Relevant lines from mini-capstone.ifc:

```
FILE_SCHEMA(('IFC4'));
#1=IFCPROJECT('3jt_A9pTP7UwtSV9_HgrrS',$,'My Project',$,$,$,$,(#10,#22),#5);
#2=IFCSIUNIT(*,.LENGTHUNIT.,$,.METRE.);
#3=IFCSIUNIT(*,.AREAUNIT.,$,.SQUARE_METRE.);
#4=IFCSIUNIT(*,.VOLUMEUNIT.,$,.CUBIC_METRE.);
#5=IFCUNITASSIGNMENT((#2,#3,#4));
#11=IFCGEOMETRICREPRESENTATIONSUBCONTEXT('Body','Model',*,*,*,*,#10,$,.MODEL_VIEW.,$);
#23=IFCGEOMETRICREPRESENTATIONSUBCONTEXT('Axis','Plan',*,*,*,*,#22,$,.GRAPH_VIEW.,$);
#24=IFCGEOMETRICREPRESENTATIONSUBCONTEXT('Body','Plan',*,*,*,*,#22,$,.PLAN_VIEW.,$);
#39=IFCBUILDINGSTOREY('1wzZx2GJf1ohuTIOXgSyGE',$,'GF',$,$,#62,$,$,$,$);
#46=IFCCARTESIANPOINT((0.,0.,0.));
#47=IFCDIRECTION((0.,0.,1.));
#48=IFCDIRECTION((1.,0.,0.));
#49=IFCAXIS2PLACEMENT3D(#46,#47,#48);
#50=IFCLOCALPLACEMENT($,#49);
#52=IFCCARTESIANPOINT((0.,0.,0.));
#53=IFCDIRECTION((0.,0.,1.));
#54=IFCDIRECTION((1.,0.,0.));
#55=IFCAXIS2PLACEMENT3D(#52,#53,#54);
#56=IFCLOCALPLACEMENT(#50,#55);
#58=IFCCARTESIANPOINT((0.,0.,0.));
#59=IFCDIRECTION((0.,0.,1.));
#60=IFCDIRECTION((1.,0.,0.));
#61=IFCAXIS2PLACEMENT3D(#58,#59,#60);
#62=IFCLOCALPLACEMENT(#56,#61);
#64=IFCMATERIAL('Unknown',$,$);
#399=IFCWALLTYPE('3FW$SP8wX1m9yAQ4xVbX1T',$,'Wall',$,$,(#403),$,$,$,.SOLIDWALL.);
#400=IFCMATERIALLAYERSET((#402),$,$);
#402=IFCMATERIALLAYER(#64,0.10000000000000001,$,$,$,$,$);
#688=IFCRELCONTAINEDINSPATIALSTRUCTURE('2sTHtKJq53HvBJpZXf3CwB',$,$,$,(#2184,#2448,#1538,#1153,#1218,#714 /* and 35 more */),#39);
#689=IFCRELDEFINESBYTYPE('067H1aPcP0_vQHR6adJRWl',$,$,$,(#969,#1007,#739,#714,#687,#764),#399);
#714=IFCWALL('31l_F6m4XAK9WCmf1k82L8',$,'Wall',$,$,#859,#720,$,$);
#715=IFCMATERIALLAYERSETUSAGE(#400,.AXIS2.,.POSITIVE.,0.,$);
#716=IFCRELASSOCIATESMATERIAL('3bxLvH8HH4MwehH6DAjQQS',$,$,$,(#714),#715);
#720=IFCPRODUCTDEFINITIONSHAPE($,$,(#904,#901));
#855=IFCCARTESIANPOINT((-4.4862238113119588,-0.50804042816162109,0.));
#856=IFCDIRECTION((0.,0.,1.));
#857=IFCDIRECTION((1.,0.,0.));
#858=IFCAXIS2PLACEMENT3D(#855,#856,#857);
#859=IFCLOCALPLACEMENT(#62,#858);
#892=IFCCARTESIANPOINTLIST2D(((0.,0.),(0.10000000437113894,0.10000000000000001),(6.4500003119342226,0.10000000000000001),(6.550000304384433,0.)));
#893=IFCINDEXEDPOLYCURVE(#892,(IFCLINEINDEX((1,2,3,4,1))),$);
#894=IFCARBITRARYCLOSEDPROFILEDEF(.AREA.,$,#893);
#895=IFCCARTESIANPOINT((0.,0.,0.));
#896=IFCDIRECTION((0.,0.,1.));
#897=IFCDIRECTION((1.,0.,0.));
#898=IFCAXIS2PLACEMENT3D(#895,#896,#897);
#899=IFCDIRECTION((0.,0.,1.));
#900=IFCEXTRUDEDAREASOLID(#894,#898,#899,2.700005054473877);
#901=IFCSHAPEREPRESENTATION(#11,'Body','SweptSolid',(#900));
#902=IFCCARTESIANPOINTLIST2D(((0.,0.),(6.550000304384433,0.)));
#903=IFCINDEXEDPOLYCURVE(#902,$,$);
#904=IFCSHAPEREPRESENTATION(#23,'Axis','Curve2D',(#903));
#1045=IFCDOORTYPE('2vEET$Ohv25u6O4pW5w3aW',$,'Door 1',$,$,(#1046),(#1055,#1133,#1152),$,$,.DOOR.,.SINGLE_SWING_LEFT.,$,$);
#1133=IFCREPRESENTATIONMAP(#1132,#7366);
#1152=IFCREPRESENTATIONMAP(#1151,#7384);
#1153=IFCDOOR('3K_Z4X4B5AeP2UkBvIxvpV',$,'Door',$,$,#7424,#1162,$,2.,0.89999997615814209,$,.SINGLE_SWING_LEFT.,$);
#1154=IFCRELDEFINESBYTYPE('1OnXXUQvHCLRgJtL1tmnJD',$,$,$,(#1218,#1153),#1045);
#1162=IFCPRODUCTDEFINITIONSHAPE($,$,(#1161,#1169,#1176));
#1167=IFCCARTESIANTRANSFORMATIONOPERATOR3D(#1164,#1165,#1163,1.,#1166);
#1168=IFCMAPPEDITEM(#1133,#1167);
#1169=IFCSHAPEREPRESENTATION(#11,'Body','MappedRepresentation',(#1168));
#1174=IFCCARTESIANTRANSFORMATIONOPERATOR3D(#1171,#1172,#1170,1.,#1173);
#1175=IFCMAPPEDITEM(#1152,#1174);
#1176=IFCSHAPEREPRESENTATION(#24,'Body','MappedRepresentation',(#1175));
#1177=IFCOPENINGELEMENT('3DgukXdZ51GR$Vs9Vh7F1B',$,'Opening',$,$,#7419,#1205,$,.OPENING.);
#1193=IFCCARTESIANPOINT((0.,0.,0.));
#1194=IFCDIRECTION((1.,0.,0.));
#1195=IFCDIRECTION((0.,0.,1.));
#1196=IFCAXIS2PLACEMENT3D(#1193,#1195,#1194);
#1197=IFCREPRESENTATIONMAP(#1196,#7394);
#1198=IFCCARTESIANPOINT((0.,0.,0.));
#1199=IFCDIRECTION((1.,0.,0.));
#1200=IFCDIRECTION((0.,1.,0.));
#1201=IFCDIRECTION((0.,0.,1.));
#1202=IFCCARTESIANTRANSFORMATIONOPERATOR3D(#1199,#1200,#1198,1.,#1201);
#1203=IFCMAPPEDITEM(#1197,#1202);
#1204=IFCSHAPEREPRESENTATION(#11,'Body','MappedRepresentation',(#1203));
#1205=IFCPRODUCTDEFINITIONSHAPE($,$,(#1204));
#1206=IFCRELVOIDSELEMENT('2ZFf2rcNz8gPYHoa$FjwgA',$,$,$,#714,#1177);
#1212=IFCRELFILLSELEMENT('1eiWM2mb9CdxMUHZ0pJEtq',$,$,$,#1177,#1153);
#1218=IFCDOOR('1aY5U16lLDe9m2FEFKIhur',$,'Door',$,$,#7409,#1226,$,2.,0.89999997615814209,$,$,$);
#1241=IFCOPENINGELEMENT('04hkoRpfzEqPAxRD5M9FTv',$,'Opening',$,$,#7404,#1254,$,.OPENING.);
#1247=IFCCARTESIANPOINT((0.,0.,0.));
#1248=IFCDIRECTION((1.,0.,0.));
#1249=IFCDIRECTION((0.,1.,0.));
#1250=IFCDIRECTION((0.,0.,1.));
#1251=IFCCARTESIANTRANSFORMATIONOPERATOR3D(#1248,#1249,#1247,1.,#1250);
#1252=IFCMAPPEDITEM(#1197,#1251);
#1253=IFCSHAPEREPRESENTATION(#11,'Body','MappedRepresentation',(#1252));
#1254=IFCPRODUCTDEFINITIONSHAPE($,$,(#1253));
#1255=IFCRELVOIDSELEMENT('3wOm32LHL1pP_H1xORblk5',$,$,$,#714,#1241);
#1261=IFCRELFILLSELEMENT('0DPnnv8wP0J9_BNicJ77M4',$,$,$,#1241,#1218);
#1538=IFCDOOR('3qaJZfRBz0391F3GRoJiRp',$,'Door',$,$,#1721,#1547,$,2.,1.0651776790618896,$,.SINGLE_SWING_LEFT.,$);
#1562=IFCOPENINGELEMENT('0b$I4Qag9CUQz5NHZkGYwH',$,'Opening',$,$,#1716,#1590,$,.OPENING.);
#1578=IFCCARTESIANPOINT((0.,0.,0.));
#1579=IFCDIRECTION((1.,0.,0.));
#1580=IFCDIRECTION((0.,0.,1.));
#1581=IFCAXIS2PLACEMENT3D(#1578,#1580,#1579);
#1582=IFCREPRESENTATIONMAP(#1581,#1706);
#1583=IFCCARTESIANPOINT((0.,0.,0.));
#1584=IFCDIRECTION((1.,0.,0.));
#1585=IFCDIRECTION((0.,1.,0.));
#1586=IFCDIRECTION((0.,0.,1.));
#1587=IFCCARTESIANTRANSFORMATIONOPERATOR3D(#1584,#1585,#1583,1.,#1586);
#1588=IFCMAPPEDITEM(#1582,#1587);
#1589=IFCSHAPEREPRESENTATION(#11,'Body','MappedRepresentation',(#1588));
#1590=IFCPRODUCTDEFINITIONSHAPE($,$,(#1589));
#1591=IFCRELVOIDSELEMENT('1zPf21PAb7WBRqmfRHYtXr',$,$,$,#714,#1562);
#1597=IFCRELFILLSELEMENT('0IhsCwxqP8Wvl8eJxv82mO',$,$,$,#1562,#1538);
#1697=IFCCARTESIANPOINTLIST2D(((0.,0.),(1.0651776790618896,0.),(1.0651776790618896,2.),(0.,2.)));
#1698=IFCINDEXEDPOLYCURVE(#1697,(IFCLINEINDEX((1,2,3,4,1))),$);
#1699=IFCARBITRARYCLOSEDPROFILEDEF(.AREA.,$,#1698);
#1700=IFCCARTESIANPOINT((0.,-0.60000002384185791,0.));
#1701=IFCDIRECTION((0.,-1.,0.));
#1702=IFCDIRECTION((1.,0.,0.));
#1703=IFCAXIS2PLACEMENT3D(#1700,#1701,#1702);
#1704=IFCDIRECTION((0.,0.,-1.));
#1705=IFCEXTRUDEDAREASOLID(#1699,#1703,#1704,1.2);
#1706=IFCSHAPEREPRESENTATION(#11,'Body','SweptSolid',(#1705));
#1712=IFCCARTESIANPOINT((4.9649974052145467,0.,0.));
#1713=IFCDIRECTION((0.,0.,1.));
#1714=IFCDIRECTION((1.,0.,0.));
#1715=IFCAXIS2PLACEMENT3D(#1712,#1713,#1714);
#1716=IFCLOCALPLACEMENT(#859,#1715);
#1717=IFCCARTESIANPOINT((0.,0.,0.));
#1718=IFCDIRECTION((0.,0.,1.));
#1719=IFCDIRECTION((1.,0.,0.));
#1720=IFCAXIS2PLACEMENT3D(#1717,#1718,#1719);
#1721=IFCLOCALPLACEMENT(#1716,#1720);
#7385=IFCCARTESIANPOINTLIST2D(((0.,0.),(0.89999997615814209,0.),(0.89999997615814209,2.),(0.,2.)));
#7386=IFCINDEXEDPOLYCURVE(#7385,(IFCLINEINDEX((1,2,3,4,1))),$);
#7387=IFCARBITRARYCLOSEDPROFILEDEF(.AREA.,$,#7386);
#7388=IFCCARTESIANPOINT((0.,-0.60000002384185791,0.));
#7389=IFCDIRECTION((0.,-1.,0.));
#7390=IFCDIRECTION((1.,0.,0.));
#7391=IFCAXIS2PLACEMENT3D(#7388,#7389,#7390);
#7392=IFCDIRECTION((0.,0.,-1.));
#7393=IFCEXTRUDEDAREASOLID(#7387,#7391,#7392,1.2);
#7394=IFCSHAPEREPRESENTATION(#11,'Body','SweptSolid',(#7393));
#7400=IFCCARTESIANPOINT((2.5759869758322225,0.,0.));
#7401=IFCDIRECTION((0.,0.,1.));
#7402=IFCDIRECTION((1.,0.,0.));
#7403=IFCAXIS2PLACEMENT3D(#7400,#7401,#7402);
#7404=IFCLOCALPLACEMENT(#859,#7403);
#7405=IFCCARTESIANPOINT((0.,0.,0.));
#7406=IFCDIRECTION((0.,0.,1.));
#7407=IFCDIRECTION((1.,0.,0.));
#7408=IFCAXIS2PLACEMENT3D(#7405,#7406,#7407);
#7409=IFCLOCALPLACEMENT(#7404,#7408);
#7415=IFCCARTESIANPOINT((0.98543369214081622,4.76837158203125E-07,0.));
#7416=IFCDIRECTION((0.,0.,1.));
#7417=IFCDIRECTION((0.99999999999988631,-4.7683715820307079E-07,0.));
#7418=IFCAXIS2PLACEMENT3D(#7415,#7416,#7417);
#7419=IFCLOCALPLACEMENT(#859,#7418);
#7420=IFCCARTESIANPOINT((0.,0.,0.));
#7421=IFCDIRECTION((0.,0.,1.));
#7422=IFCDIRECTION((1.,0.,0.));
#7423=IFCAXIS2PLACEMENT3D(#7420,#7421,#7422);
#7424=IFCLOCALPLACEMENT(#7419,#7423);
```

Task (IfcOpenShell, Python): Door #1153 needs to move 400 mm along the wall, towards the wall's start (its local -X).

```python
import ifcopenshell
import ifcopenshell.api.geometry
import ifcopenshell.util.placement
import ifcopenshell.util.unit

model = ifcopenshell.open("mini-capstone.ifc")
unit_scale = ifcopenshell.util.unit.calculate_unit_scale(model)

door = model.by_guid("3K_Z4X4B5AeP2UkBvIxvpV")
opening = door.FillsVoids[0].RelatingOpeningElement
wall = opening.VoidsElements[0].RelatingBuildingElement

wall_matrix = ifcopenshell.util.placement.get_local_placement(wall.ObjectPlacement)
shift = wall_matrix[:3, 0] * -0.4 / unit_scale
before = ifcopenshell.util.placement.get_local_placement(door.ObjectPlacement)[:3, 3].copy()

# The door is placed relative to its opening, so it follows when the opening moves.
matrix = ifcopenshell.util.placement.get_local_placement(opening.ObjectPlacement)
matrix[:3, 3] += shift
ifcopenshell.api.geometry.edit_object_placement(
    model, product=opening, matrix=matrix, is_si=False, should_transform_children=True
)

after = ifcopenshell.util.placement.get_local_placement(door.ObjectPlacement)[:3, 3]
print("door moved by", (after - before).round(3) + 0.0)

model.write("mini-capstone-out.ifc")
```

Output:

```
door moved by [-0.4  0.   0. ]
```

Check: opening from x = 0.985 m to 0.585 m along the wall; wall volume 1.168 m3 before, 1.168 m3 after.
